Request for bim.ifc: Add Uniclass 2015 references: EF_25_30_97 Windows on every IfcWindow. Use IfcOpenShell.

First a look at what the model holds.

```python
import ifcopenshell

model = ifcopenshell.open("bim.ifc")
print(model.schema)
print("classifications:", [c.Name for c in model.by_type("IfcClassification")])
for ifc_class in ("IfcDoor", "IfcRoof", "IfcStair", "IfcWall", "IfcWindow"):
    print(ifc_class, len(model.by_type(ifc_class)))
```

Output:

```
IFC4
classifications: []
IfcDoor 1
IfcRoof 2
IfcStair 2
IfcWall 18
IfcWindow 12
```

```python
import ifcopenshell
import ifcopenshell.api.classification

model = ifcopenshell.open("bim.ifc")

system = ifcopenshell.api.classification.add_classification(model, classification="Uniclass 2015")

codes = {
    "IfcWindow": ("EF_25_30_97", "Windows"),
}
for ifc_class, (code, name) in codes.items():
    products = model.by_type(ifc_class)
    ifcopenshell.api.classification.add_reference(
        model, products=products, classification=system, identification=code, name=name
    )
    print(code, len(products))

model.write("bim-out.ifc")
```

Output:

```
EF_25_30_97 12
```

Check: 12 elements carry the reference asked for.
